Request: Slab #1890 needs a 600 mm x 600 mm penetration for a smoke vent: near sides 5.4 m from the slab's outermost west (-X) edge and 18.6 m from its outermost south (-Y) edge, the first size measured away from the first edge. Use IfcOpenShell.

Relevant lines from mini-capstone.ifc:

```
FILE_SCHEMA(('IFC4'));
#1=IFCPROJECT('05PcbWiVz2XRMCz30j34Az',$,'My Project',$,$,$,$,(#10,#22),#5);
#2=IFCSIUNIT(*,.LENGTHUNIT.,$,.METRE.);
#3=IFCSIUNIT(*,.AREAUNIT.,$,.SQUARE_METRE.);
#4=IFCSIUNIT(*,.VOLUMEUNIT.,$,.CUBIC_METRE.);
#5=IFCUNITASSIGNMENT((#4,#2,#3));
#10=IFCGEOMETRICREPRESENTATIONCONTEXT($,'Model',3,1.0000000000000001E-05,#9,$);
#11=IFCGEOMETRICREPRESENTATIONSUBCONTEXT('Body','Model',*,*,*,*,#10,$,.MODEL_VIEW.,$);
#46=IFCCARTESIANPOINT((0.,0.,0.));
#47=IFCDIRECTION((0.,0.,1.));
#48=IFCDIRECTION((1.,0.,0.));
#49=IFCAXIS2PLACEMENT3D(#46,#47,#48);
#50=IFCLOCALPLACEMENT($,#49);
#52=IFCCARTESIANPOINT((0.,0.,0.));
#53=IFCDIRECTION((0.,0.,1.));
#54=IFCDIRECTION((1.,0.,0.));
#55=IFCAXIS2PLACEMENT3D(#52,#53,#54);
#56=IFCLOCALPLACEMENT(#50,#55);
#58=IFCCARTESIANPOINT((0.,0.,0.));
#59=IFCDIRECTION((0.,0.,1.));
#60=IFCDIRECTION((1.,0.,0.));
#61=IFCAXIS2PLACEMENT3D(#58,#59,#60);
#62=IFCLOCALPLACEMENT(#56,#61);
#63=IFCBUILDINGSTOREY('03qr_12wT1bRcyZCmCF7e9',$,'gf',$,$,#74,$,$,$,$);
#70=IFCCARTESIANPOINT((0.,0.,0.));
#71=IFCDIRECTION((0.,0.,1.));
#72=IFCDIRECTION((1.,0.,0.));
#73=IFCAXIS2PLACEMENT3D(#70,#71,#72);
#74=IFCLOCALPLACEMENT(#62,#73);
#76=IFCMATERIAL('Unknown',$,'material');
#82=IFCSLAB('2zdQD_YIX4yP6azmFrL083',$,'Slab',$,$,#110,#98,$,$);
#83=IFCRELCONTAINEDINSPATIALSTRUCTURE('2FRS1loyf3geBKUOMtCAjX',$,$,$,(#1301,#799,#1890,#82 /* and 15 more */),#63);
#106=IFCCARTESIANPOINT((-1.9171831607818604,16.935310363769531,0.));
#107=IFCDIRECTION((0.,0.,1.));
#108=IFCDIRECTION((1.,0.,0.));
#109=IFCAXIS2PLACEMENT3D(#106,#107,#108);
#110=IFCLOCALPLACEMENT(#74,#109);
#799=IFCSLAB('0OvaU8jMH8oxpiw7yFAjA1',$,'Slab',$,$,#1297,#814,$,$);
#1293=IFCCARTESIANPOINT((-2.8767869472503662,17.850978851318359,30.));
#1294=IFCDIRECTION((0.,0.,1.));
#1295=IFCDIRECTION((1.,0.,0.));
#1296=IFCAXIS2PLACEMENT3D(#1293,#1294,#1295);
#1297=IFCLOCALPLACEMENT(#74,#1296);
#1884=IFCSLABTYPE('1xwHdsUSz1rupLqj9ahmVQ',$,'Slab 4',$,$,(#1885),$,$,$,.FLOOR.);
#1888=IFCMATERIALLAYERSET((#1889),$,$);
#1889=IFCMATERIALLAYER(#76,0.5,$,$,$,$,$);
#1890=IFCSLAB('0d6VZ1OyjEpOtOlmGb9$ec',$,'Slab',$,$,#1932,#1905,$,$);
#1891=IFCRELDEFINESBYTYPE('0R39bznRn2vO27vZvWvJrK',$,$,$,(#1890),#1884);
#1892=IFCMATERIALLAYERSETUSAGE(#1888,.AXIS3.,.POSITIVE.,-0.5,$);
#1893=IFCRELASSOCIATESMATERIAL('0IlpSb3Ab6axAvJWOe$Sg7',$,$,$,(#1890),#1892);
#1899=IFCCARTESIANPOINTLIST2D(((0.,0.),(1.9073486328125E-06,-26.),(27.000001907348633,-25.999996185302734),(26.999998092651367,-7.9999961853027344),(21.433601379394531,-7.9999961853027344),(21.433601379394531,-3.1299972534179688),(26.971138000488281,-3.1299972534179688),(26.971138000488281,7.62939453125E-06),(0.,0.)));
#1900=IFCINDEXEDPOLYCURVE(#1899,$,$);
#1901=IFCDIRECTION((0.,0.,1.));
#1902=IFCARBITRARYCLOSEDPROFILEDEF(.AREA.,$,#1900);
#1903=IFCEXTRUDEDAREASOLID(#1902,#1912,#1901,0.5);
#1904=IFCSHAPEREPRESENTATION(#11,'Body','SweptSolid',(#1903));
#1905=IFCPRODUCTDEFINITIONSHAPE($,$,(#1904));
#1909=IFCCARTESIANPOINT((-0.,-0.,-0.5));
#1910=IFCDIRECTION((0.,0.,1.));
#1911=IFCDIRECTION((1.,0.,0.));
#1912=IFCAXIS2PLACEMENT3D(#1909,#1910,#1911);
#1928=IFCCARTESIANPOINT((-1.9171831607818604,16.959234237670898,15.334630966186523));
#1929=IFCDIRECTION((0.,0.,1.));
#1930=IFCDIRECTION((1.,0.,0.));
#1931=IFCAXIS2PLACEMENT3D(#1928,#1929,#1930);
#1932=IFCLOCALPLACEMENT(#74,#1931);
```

```python
import numpy as np
import ifcopenshell
import ifcopenshell.api.feature
import ifcopenshell.api.geometry
import ifcopenshell.api.root
import ifcopenshell.geom
import ifcopenshell.util.placement
import ifcopenshell.util.representation
import ifcopenshell.util.shape
import ifcopenshell.util.unit

model = ifcopenshell.open("mini-capstone.ifc")
unit_scale = ifcopenshell.util.unit.calculate_unit_scale(model)
settings = ifcopenshell.geom.settings()


def volume(element):
    """Net volume in cubic metres, openings subtracted."""
    shape = ifcopenshell.geom.create_shape(settings, element)
    return ifcopenshell.util.shape.get_volume(shape.geometry)


slab = model.by_guid("0d6VZ1OyjEpOtOlmGb9$ec")
before = volume(slab)

# Extent in the slab's own axes, in metres. The edges named are its -X and -Y sides.
slab_shape = ifcopenshell.geom.create_shape(settings, slab)
vertices = ifcopenshell.util.shape.get_vertices(slab_shape.geometry)
x_min, y_min, bottom = vertices.min(axis=0)
top = vertices[:, 2].max()

opening = ifcopenshell.api.root.create_entity(model, ifc_class="IfcOpeningElement", name="Smoke vent opening", predefined_type="OPENING")
context = ifcopenshell.util.representation.get_context(model, "Model", "Body", "MODEL_VIEW")
width, depth = 0.6, 0.6
outline = [(0.0, 0.0), (width, 0.0), (width, depth), (0.0, depth), (0.0, 0.0)]
# Overshoot both faces by 50 mm so the cut is clean.
shape = ifcopenshell.api.geometry.add_slab_representation(
    model, context=context, depth=top - bottom + 0.1, polyline=outline
)
ifcopenshell.api.geometry.assign_representation(model, product=opening, representation=shape)

matrix = ifcopenshell.util.placement.get_local_placement(slab.ObjectPlacement)
matrix[:, 3] = matrix @ np.append(np.array([x_min + 5.4, y_min + 18.6, bottom - 0.05]) / unit_scale, 1.0)
ifcopenshell.api.geometry.edit_object_placement(model, product=opening, matrix=matrix, is_si=False)
ifcopenshell.api.feature.add_feature(model, feature=opening, element=slab)

after = volume(slab)

print(f"slab volume {before:.3f} -> {after:.3f} m3")

model.write("mini-capstone-out.ifc")
```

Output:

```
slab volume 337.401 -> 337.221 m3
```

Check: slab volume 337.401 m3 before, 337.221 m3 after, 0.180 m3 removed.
